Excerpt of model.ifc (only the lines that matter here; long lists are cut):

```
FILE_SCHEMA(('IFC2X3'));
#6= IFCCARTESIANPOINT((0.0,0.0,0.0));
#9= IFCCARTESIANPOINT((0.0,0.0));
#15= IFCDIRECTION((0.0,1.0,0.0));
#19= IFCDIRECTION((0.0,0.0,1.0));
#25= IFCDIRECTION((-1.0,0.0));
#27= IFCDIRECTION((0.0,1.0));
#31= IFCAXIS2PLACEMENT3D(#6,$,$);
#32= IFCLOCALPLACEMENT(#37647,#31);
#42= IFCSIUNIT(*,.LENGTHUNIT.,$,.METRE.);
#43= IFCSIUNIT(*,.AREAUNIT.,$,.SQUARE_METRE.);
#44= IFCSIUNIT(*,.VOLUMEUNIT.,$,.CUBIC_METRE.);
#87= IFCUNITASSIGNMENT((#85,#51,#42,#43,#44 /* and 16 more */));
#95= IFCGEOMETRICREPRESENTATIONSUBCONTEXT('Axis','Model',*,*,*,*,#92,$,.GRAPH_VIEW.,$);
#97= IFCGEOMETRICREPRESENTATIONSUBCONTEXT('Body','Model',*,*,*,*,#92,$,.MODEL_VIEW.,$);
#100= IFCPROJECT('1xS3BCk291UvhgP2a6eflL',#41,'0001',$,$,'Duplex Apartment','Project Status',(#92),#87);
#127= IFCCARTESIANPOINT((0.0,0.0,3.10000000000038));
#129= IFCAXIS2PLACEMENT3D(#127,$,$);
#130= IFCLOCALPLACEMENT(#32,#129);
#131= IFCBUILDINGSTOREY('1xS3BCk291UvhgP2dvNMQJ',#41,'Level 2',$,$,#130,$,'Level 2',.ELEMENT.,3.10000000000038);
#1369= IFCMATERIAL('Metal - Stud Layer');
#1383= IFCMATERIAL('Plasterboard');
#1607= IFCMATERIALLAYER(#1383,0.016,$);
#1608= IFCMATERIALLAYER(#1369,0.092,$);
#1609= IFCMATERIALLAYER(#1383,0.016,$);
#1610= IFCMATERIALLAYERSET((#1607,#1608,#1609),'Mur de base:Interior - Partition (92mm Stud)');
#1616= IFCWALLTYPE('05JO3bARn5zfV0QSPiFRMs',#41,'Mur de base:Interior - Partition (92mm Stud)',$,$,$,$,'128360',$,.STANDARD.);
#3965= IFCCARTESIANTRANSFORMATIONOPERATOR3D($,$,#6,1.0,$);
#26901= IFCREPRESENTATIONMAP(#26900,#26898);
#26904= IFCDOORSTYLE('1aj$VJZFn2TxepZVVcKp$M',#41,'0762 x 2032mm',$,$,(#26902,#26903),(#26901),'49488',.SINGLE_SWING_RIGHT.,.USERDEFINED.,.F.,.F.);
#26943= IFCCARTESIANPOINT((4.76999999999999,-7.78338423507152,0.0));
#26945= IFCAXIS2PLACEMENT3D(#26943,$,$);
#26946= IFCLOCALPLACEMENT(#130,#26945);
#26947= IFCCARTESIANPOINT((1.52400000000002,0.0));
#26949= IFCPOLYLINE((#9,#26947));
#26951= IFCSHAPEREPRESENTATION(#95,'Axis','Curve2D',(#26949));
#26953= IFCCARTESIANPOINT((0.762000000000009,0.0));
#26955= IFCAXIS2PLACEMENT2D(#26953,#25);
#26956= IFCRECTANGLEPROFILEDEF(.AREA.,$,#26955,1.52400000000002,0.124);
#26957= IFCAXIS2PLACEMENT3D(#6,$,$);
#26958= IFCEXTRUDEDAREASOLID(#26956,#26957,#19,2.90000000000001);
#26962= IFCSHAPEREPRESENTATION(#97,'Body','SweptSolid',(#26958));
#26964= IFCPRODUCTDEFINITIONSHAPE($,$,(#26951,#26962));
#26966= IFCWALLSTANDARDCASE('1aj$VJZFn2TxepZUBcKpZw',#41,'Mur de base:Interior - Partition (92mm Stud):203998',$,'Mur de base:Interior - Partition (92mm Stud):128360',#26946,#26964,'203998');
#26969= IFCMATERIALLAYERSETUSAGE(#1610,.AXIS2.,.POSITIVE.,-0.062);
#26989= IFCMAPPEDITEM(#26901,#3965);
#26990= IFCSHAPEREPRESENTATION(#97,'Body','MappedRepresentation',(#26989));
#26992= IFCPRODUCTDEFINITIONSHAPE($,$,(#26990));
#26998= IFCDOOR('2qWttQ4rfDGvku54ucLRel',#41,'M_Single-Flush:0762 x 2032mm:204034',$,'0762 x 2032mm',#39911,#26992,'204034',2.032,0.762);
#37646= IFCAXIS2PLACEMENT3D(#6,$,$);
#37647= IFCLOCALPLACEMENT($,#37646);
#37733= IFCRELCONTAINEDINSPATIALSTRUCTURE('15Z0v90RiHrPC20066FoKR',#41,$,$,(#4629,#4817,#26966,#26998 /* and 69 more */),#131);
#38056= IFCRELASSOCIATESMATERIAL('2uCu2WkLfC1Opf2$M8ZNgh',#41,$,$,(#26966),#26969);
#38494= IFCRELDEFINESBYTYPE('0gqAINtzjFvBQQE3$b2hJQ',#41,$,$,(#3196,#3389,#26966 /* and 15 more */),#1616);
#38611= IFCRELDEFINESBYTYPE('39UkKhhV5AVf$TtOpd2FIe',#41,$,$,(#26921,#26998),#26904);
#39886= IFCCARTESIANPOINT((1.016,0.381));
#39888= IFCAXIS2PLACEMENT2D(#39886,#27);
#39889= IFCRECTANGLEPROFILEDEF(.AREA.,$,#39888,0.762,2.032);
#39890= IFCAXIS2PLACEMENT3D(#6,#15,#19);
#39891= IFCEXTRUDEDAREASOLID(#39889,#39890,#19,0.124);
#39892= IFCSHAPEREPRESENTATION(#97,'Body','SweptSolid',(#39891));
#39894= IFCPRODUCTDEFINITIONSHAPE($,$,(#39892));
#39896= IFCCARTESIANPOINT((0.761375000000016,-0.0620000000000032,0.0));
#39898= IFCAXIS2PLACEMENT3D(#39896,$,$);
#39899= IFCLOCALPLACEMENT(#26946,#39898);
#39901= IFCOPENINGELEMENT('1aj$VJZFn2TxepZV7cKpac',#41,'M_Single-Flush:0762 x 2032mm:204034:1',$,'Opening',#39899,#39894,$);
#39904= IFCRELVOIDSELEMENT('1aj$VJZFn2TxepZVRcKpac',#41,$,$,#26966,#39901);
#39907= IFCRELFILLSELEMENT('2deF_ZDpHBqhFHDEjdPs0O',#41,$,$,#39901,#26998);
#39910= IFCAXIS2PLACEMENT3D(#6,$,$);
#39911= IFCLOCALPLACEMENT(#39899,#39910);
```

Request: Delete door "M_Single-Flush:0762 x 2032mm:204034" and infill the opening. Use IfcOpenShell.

```python
import ifcopenshell
import ifcopenshell.api.feature
import ifcopenshell.api.root
import ifcopenshell.geom
import ifcopenshell.util.shape

model = ifcopenshell.open("model.ifc")
settings = ifcopenshell.geom.settings()


def volume(element):
    """Net volume in cubic metres, openings subtracted."""
    shape = ifcopenshell.geom.create_shape(settings, element)
    return ifcopenshell.util.shape.get_volume(shape.geometry)


door = model.by_id(26998)
opening = door.FillsVoids[0].RelatingOpeningElement
wall = opening.VoidsElements[0].RelatingBuildingElement
before = volume(wall)

ifcopenshell.api.root.remove_product(model, product=door)
ifcopenshell.api.feature.remove_feature(model, feature=opening)

after = volume(wall)

print(f"wall volume {before:.3f} -> {after:.3f} m3")

model.write("model_updated.ifc")
```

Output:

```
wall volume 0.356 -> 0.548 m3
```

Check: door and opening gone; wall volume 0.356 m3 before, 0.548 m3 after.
